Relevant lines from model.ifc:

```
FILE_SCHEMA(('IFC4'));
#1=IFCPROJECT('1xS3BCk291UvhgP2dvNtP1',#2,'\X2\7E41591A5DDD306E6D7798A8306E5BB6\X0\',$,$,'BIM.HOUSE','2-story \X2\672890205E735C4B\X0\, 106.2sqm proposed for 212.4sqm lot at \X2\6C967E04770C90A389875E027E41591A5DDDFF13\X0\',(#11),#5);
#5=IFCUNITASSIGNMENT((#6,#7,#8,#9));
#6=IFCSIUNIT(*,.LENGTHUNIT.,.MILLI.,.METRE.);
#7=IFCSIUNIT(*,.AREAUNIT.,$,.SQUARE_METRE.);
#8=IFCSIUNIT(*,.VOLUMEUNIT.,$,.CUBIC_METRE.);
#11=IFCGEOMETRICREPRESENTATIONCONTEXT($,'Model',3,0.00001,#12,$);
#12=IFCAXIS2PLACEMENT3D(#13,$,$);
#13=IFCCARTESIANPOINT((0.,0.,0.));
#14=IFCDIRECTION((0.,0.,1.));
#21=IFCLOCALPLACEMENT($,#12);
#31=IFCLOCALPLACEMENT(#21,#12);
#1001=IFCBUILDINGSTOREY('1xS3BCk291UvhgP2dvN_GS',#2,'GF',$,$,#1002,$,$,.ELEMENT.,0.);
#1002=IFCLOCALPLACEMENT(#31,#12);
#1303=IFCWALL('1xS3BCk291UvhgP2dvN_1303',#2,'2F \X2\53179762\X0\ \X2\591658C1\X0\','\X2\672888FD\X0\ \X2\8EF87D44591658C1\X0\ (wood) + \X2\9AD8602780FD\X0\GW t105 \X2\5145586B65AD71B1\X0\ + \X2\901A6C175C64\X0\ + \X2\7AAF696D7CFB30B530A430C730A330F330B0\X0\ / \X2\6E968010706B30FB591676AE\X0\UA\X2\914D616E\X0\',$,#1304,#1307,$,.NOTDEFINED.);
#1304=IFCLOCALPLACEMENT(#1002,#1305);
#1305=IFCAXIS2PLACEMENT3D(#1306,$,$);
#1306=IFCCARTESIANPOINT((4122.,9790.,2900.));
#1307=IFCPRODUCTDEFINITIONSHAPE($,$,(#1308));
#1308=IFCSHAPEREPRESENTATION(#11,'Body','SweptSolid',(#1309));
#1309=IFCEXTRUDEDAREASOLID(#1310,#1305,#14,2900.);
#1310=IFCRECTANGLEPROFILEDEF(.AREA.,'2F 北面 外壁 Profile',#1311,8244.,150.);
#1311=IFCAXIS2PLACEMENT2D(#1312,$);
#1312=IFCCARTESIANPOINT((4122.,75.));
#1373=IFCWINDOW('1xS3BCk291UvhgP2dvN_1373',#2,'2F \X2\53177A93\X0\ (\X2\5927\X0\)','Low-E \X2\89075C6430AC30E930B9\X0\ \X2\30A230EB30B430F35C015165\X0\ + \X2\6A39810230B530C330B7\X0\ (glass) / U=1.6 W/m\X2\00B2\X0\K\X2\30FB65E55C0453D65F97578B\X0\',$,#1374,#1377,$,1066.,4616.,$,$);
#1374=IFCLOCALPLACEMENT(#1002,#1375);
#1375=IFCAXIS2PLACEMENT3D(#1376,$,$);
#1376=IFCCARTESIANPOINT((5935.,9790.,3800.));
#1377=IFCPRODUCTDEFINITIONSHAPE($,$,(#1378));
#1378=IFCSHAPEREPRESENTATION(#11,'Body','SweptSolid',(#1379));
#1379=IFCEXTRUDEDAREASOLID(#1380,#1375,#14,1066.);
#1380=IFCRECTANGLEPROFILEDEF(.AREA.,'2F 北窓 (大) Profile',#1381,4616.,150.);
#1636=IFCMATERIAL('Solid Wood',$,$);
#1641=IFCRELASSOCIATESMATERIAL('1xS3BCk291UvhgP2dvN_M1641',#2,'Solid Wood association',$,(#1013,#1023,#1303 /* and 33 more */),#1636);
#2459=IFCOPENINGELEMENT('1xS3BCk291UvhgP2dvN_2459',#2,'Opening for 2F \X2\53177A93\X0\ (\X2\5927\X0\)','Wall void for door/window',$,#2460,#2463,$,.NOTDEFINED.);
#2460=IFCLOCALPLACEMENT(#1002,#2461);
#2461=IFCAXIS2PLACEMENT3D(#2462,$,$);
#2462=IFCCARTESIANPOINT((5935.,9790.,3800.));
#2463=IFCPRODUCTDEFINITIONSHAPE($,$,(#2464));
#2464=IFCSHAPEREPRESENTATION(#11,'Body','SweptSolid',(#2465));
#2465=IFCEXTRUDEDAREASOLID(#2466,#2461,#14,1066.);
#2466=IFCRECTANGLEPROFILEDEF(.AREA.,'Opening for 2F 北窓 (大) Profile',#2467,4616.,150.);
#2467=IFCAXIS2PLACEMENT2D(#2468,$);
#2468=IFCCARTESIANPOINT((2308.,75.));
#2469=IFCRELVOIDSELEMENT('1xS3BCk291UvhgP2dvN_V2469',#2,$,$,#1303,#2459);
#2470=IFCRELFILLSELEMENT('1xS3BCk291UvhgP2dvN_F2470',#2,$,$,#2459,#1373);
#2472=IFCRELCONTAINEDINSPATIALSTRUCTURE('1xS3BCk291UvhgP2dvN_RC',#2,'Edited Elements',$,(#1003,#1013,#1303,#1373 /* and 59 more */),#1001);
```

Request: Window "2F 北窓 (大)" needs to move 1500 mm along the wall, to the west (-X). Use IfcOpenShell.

```python
import ifcopenshell
import ifcopenshell.api.geometry
import ifcopenshell.util.placement
import ifcopenshell.util.unit

model = ifcopenshell.open("model.ifc")
unit_scale = ifcopenshell.util.unit.calculate_unit_scale(model)

window = model.by_guid("1xS3BCk291UvhgP2dvN_1373")
opening = window.FillsVoids[0].RelatingOpeningElement
wall = opening.VoidsElements[0].RelatingBuildingElement

wall_matrix = ifcopenshell.util.placement.get_local_placement(wall.ObjectPlacement)
shift = wall_matrix[:3, 0] * -1.5 / unit_scale
before = ifcopenshell.util.placement.get_local_placement(window.ObjectPlacement)[:3, 3].copy()

# The window is not placed relative to its opening, so move both.
for product in (opening, window):
    matrix = ifcopenshell.util.placement.get_local_placement(product.ObjectPlacement)
    matrix[:3, 3] += shift
    ifcopenshell.api.geometry.edit_object_placement(model, product=product, matrix=matrix, is_si=False)

after = ifcopenshell.util.placement.get_local_placement(window.ObjectPlacement)[:3, 3]
print("window moved by", (after - before).round(3) + 0.0)

model.write("model_updated.ifc")
```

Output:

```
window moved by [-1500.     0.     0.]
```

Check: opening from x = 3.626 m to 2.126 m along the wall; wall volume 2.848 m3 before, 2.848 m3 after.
